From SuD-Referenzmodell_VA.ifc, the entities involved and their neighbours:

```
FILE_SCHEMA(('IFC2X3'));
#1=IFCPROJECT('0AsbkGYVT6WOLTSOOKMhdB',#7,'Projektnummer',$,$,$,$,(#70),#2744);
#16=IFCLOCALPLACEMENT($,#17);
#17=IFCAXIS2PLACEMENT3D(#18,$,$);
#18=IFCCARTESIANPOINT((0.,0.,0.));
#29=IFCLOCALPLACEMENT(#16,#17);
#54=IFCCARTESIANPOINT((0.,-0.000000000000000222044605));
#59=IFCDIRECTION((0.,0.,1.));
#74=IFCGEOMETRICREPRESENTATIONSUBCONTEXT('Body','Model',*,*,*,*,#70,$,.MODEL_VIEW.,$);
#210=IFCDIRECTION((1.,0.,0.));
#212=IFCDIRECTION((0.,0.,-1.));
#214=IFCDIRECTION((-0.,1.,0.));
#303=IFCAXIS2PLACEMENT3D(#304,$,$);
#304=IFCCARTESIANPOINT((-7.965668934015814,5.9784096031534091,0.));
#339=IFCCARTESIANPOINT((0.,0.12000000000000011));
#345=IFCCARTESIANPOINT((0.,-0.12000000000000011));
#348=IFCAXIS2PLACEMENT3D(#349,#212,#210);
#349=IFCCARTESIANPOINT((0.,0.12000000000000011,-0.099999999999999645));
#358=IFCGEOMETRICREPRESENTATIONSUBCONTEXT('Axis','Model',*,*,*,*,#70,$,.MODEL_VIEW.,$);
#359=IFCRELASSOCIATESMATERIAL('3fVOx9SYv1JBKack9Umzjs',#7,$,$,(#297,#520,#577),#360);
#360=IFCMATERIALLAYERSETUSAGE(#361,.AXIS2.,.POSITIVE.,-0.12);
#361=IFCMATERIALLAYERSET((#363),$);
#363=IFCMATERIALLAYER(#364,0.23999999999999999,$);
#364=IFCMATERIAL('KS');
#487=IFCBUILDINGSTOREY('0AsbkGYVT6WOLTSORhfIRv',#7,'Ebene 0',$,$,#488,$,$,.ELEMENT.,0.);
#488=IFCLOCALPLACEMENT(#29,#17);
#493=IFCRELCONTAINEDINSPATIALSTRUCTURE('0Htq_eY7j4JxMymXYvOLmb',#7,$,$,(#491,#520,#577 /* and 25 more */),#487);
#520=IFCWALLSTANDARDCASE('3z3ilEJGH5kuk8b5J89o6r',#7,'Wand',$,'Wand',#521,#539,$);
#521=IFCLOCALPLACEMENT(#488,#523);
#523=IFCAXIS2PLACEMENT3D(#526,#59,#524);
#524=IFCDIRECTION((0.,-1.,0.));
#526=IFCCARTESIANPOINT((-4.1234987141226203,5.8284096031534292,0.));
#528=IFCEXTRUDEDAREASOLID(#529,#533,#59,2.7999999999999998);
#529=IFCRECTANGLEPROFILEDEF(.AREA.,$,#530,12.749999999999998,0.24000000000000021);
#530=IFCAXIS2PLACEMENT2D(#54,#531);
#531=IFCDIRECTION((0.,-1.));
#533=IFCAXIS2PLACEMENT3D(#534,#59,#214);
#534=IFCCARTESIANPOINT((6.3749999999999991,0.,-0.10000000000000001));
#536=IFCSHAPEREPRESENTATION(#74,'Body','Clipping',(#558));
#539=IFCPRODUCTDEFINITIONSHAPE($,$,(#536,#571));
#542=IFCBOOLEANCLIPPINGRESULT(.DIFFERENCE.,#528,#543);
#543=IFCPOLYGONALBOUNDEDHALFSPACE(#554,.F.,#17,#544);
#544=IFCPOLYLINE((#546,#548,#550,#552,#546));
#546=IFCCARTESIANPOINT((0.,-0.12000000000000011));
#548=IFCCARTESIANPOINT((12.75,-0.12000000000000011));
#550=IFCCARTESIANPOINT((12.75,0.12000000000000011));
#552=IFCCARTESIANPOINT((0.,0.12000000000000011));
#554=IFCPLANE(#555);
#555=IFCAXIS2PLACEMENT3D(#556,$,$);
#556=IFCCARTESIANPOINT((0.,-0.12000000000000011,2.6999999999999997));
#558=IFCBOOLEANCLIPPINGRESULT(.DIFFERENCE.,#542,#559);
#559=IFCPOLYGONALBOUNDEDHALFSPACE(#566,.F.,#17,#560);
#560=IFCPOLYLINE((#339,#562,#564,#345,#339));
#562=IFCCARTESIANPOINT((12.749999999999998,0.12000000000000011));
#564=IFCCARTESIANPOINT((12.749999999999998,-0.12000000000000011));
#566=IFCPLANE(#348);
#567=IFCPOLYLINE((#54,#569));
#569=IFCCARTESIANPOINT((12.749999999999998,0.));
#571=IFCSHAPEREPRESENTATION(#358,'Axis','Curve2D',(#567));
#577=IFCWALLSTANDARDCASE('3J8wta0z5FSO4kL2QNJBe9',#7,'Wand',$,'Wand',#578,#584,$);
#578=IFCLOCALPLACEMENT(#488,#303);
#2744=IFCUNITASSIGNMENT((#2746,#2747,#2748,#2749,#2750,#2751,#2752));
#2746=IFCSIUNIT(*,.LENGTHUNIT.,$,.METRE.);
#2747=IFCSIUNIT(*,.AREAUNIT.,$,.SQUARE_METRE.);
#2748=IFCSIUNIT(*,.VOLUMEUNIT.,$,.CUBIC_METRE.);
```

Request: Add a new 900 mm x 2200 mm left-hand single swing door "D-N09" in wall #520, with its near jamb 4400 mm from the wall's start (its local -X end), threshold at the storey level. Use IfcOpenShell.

```python
import numpy as np
import ifcopenshell
import ifcopenshell.api.feature
import ifcopenshell.api.geometry
import ifcopenshell.api.root
import ifcopenshell.api.spatial
import ifcopenshell.api.type
import ifcopenshell.geom
import ifcopenshell.util.element
import ifcopenshell.util.placement
import ifcopenshell.util.representation
import ifcopenshell.util.shape
import ifcopenshell.util.unit

model = ifcopenshell.open("SuD-Referenzmodell_VA.ifc")
unit_scale = ifcopenshell.util.unit.calculate_unit_scale(model)
settings = ifcopenshell.geom.settings()


def volume(element):
    """Net volume in cubic metres, openings subtracted."""
    shape = ifcopenshell.geom.create_shape(settings, element)
    return ifcopenshell.util.shape.get_volume(shape.geometry)


wall = model.by_id(520)
storey = ifcopenshell.util.element.get_container(wall, ifc_class="IfcBuildingStorey")
context = ifcopenshell.util.representation.get_context(model, "Model", "Body", "MODEL_VIEW")
before = volume(wall)

width, height, from_end, sill = 0.9, 2.2, 4.4, 0.0  # metres

# The wall runs along its own X axis, and the end named is its -X end.
wall_shape = ifcopenshell.geom.create_shape(settings, wall)
x, y, z = ifcopenshell.util.shape.get_vertices(wall_shape.geometry).T
start = x.min() + from_end
face, thickness = float(y.min()), float(y.max() - y.min())
wall_matrix = ifcopenshell.util.placement.get_local_placement(wall.ObjectPlacement)
level = ifcopenshell.util.placement.get_local_placement(storey.ObjectPlacement)[2, 3]


def in_wall(x, y):
    """Placement at x, y metres in the wall's axes, at sill height."""
    matrix = wall_matrix.copy()
    matrix[:, 3] = wall_matrix @ np.array([x / unit_scale, y / unit_scale, 0.0, 1.0])
    matrix[2, 3] = level + sill / unit_scale
    return matrix


# Opening: a box that overshoots both wall faces by 50 mm.
opening = ifcopenshell.api.root.create_entity(model, ifc_class="IfcOpeningElement")
box = ifcopenshell.api.geometry.add_wall_representation(
    model, context=context, length=width, height=height, thickness=thickness + 0.1
)
ifcopenshell.api.geometry.assign_representation(model, product=opening, representation=box)
ifcopenshell.api.geometry.edit_object_placement(model, product=opening, matrix=in_wall(start, face - 0.05), is_si=False)
ifcopenshell.api.feature.add_feature(model, feature=opening, element=wall)

door = ifcopenshell.api.root.create_entity(model, ifc_class="IfcDoor", name="D-N09")
door.OverallWidth, door.OverallHeight = width / unit_scale, height / unit_scale
body = ifcopenshell.api.geometry.add_door_representation(
    model,
    context=context,
    overall_width=door.OverallWidth,
    overall_height=door.OverallHeight,
    operation_type="SINGLE_SWING_LEFT",
    lining_properties={"LiningDepth": thickness / unit_scale, "ThresholdDepth": thickness / unit_scale},
)
ifcopenshell.api.geometry.assign_representation(model, product=door, representation=body)
ifcopenshell.api.spatial.assign_container(model, products=[door], relating_structure=storey)
fills = ifcopenshell.api.feature.add_filling(model, opening=opening, element=door)
fills.OwnerHistory = door.OwnerHistory  # required in IFC2X3

# IFC2X3 keeps the operation on the door style.
style = ifcopenshell.api.root.create_entity(model, ifc_class="IfcDoorStyle", name="D-N09")
style.OperationType, style.ConstructionType = "SINGLE_SWING_LEFT", "NOTDEFINED"
style.ParameterTakesPrecedence = style.Sizeable = False
ifcopenshell.api.type.assign_type(model, related_objects=[door], relating_type=style)

# The lining spans the wall, so the door starts at the wall face.
ifcopenshell.api.geometry.edit_object_placement(model, product=door, matrix=in_wall(start, face), is_si=False)

after = volume(wall)

print(f"wall volume {before:.3f} -> {after:.3f} m3")

model.write("SuD-Referenzmodell_VA_updated.ifc")
```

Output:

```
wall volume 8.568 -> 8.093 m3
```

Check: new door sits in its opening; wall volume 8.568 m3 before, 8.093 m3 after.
